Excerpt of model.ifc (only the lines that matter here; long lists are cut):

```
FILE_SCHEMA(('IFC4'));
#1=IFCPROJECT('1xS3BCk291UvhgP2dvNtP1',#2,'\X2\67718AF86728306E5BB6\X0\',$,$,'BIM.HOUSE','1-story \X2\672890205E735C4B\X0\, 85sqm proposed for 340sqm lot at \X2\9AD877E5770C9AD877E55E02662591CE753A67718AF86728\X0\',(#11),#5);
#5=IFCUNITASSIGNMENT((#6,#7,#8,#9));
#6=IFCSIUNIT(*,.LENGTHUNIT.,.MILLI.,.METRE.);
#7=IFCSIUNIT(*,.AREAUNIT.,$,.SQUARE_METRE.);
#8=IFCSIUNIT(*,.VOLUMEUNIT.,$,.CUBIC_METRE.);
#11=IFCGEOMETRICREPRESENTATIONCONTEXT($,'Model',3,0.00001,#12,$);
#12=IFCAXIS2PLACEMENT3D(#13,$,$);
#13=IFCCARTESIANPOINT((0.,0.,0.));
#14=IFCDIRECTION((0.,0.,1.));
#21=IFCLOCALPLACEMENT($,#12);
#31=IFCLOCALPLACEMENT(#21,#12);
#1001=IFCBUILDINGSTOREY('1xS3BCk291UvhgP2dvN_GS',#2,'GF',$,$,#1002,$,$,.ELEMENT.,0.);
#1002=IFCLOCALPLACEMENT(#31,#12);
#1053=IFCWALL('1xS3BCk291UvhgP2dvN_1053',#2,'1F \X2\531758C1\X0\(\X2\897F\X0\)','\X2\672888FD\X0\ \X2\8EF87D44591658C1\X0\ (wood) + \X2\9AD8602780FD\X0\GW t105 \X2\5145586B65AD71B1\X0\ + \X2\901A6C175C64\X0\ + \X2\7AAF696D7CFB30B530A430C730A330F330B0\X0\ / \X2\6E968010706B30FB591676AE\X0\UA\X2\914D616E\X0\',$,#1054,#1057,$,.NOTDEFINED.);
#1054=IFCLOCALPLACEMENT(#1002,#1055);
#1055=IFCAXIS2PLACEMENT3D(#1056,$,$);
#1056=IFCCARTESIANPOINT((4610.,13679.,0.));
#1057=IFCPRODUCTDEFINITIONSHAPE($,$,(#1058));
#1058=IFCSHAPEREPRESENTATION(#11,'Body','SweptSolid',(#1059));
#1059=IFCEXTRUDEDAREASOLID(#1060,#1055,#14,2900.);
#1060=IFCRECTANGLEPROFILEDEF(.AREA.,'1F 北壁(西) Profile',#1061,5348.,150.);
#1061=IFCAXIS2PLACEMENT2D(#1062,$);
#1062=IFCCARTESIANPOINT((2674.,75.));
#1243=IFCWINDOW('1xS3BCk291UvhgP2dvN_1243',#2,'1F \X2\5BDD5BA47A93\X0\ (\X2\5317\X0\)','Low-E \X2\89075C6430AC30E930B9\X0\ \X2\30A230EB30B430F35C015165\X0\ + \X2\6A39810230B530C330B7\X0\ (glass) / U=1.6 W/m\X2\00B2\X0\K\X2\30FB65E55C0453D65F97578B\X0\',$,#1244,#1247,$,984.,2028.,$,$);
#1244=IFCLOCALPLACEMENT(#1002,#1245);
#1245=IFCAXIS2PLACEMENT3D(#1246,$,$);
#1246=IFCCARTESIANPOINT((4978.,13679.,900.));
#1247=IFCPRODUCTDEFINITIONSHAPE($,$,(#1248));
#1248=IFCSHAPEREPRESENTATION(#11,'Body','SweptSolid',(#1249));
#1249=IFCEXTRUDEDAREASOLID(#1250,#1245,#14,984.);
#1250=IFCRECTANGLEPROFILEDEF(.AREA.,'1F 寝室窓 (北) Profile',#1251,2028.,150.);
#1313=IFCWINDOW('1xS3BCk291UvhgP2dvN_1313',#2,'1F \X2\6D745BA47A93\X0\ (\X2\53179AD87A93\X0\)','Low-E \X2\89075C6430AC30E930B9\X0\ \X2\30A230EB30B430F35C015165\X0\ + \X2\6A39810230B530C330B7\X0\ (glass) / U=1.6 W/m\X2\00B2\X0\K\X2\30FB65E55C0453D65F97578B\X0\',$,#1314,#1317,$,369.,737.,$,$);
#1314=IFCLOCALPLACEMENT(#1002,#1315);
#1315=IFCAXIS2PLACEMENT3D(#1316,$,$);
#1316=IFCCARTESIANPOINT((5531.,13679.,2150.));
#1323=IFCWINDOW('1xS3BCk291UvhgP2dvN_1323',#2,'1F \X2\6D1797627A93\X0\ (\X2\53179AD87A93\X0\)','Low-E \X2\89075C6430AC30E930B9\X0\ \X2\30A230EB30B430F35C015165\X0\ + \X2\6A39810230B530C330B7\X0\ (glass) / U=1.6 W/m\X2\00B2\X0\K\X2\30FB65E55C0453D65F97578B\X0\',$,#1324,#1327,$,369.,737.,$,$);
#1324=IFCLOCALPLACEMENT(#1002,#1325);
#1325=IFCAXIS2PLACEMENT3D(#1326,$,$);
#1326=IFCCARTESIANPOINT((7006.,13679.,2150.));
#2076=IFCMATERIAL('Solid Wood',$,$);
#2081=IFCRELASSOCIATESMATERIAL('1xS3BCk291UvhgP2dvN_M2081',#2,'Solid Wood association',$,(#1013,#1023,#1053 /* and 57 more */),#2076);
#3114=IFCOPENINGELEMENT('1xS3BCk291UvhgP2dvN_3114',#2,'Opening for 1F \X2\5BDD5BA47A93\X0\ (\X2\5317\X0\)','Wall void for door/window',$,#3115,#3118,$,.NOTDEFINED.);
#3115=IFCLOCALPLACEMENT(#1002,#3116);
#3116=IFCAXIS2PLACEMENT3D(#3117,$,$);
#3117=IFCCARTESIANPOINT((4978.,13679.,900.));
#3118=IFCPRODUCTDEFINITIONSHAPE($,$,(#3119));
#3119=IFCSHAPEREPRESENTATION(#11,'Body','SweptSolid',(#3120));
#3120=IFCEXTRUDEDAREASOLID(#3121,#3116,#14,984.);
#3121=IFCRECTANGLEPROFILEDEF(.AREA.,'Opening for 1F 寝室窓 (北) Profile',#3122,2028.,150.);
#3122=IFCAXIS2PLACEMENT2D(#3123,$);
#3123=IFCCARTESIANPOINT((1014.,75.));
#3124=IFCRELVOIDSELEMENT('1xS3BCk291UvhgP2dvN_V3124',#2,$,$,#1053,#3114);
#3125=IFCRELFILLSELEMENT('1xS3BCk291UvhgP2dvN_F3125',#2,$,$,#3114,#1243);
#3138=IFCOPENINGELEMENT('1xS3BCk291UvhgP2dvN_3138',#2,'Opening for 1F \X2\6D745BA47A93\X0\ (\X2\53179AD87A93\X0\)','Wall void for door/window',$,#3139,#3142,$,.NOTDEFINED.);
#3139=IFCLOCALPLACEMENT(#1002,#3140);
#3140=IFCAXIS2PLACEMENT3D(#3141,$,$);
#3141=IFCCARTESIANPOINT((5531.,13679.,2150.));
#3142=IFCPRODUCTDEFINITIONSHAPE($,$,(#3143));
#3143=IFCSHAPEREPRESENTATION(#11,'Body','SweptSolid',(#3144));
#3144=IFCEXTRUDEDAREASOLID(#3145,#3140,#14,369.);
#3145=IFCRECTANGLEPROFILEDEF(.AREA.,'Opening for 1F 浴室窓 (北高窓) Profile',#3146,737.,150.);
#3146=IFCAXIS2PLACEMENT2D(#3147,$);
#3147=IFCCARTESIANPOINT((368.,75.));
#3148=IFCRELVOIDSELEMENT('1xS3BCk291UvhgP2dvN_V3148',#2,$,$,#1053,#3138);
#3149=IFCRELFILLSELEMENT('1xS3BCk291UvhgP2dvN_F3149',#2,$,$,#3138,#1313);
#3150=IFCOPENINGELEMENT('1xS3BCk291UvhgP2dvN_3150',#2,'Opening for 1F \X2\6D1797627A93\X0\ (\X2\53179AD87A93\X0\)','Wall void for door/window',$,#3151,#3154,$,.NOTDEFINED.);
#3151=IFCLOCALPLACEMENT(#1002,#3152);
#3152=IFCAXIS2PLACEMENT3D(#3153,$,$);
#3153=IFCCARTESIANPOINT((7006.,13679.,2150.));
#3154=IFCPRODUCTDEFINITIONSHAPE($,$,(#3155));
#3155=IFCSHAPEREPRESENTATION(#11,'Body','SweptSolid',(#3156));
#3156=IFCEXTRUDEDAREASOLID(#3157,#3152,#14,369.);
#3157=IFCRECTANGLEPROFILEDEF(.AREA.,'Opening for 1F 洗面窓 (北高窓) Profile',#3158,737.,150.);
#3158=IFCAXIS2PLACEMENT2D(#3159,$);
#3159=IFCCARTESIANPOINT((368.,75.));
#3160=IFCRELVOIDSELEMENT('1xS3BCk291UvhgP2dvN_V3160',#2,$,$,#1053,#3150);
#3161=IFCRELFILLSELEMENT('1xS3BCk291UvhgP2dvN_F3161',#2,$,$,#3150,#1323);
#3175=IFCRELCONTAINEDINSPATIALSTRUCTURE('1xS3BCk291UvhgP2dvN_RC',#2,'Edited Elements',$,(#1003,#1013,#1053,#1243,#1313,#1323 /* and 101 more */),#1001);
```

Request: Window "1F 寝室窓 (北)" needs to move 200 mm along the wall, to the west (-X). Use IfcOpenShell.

```python
import ifcopenshell
import ifcopenshell.api.geometry
import ifcopenshell.util.placement

model = ifcopenshell.open("model.ifc")

window = model.by_guid("1xS3BCk291UvhgP2dvN_1243")
opening = window.FillsVoids[0].RelatingOpeningElement
wall = opening.VoidsElements[0].RelatingBuildingElement

wall_matrix = ifcopenshell.util.placement.get_local_placement(wall.ObjectPlacement)
shift = wall_matrix[:3, 0] * -200.0
before = ifcopenshell.util.placement.get_local_placement(window.ObjectPlacement)[:3, 3].copy()

# The window is not placed relative to its opening, so move both.
for product in (opening, window):
    matrix = ifcopenshell.util.placement.get_local_placement(product.ObjectPlacement)
    matrix[:3, 3] += shift
    ifcopenshell.api.geometry.edit_object_placement(model, product=product, matrix=matrix, is_si=False)

after = ifcopenshell.util.placement.get_local_placement(window.ObjectPlacement)[:3, 3]
print("window moved by", (after - before).round(3) + 0.0)

model.write("model_rev.ifc")
```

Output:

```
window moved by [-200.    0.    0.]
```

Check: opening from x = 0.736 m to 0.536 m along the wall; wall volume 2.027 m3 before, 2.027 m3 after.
